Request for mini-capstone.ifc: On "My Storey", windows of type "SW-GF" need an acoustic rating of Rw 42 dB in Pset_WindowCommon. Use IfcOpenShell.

First a look at what the model holds.

```python
import ifcopenshell
import ifcopenshell.util.element

model = ifcopenshell.open("mini-capstone.ifc")
print(model.schema)
storey = next(s for s in model.by_type("IfcBuildingStorey") if s.Name == "My Storey")
windows = [e for e in ifcopenshell.util.element.get_decomposition(storey) if e.is_a("IfcWindow")]
seen = {}
for e in windows:
    element_type = ifcopenshell.util.element.get_type(e)
    key = (element_type.Name if element_type != e and element_type else None, ifcopenshell.util.element.get_pset(e, "Pset_WindowCommon", "AcousticRating"))
    seen[key] = seen.get(key, 0) + 1
for (name, value), count in sorted(seen.items(), key=str):
    print(count, "x", name, "|", value)
```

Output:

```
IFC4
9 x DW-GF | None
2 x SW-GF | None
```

```python
import ifcopenshell
import ifcopenshell.api.pset
import ifcopenshell.util.element

model = ifcopenshell.open("mini-capstone.ifc")

storey = next(s for s in model.by_type("IfcBuildingStorey") if s.Name == "My Storey")
windows = [e for e in ifcopenshell.util.element.get_decomposition(storey) if e.is_a("IfcWindow")]

count = 0
for e in windows:
    element_type = ifcopenshell.util.element.get_type(e)
    if element_type in (None, e) or element_type.Name != "SW-GF":
        continue
    # add_pset returns the element's existing set when there is one.
    pset = ifcopenshell.api.pset.add_pset(model, product=e, name="Pset_WindowCommon")
    ifcopenshell.api.pset.edit_pset(model, pset=pset, properties={"AcousticRating": "Rw 42 dB"})
    count += 1

print(count, "windows updated")

model.write("mini-capstone_updated.ifc")
```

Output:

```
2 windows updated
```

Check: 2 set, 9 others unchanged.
